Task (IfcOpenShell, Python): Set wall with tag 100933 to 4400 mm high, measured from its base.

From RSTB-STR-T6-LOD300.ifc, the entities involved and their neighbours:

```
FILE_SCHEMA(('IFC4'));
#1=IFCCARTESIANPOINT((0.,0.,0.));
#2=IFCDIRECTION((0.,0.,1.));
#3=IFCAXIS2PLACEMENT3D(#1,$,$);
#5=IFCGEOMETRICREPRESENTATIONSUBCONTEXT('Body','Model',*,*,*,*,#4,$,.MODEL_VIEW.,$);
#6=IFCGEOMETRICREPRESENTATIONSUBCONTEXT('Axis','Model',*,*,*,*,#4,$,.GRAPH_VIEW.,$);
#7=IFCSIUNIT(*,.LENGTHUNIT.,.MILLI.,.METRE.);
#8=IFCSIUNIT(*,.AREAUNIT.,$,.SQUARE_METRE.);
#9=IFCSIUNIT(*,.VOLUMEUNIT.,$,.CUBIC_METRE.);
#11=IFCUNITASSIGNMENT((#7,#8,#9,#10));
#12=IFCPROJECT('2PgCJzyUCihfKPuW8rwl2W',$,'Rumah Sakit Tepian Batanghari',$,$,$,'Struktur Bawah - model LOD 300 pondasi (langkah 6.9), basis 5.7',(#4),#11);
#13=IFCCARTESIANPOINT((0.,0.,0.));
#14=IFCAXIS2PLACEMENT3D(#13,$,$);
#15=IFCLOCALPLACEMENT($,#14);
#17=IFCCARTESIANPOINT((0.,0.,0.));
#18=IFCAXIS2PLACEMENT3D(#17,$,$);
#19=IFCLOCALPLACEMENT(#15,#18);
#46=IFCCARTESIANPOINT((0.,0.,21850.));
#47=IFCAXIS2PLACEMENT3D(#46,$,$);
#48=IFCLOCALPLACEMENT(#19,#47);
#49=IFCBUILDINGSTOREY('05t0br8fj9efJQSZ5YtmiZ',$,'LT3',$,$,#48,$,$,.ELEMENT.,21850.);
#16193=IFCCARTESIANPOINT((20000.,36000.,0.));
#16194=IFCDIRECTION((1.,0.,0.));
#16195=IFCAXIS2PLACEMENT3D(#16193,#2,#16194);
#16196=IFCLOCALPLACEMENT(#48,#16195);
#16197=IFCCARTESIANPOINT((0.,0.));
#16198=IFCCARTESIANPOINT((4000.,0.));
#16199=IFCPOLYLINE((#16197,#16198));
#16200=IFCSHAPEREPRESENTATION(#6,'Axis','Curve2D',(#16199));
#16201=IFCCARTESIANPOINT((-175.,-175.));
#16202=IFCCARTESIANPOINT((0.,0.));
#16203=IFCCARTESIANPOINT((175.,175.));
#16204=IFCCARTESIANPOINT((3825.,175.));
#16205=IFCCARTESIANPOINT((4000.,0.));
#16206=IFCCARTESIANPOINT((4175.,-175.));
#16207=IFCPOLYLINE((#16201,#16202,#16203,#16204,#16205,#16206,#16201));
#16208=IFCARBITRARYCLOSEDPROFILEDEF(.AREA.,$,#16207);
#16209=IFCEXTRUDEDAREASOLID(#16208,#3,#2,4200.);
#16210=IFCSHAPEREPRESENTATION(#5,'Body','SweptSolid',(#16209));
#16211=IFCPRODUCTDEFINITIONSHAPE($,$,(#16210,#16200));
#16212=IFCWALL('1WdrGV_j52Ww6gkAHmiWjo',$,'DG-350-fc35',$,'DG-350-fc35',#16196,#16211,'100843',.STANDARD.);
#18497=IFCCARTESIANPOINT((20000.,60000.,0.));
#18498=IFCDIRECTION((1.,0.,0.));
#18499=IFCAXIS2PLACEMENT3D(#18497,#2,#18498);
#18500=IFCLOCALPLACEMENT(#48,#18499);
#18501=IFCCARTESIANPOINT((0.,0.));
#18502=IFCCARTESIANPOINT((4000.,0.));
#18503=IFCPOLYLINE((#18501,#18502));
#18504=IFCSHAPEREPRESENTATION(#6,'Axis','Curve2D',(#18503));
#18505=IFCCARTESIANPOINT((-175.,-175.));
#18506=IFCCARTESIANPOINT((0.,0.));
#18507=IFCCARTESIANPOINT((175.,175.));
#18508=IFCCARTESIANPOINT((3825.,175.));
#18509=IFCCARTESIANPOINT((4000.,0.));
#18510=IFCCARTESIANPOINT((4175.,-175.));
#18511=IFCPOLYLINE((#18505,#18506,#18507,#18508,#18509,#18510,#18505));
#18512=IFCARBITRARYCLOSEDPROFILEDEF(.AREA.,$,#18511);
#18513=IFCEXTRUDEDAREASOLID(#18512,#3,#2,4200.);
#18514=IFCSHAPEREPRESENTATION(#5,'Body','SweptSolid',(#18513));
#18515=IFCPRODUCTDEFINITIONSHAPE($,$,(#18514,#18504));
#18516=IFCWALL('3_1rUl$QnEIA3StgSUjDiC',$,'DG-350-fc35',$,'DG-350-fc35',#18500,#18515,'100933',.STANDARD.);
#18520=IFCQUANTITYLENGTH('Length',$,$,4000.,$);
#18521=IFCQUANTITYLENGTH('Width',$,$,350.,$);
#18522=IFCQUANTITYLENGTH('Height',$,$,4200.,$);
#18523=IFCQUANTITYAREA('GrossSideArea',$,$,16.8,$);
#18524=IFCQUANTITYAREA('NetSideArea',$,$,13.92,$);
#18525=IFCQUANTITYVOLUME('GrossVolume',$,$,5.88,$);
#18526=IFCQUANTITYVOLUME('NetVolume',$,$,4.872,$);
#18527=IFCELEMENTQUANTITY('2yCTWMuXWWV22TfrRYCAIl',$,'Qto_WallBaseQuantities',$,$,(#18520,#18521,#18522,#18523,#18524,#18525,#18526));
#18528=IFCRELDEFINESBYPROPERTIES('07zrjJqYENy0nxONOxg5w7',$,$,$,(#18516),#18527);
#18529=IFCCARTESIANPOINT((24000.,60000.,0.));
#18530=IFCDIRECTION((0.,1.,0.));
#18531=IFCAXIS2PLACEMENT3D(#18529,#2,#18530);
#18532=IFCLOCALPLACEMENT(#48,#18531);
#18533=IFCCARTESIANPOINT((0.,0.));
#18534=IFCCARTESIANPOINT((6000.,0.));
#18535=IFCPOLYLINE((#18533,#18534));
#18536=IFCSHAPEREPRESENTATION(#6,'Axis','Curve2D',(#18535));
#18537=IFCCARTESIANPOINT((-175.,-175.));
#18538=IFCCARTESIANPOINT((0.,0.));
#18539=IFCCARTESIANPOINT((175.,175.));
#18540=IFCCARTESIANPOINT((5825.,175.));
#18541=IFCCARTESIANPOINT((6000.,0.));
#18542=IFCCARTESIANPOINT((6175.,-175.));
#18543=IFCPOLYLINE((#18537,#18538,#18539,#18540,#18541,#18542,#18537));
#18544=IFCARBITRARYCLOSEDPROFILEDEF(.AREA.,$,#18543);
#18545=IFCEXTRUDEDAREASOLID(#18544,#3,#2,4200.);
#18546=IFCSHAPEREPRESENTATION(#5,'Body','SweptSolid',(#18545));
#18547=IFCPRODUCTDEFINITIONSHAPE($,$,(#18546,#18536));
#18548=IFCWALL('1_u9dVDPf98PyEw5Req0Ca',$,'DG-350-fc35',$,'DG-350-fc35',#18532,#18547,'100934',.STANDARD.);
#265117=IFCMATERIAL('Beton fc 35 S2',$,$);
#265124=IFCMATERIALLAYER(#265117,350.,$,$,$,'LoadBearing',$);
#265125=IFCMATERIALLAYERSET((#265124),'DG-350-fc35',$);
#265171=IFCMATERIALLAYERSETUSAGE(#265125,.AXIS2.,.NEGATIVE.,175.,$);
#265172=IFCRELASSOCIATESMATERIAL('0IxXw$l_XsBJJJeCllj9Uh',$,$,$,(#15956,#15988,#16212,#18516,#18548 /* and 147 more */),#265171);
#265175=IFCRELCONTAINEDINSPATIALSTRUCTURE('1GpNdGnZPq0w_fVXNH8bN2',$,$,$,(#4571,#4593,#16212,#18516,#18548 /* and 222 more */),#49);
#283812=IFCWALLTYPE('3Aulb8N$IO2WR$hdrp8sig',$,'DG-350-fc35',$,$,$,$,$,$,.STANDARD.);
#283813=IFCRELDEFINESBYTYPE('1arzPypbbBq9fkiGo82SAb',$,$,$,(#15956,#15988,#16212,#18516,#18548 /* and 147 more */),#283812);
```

```python
import ifcopenshell
import ifcopenshell.api.pset
import ifcopenshell.geom
import ifcopenshell.util.element
import ifcopenshell.util.representation
import ifcopenshell.util.shape
import ifcopenshell.util.unit

model = ifcopenshell.open("RSTB-STR-T6-LOD300.ifc")
unit_scale = ifcopenshell.util.unit.calculate_unit_scale(model)
area_scale = ifcopenshell.util.unit.calculate_unit_scale(model, "AREAUNIT")
volume_scale = ifcopenshell.util.unit.calculate_unit_scale(model, "VOLUMEUNIT")
settings = ifcopenshell.geom.settings()


def volume(element):
    """Net volume in cubic metres, openings subtracted."""
    shape = ifcopenshell.geom.create_shape(settings, element)
    return ifcopenshell.util.shape.get_volume(shape.geometry)


wall = model.by_id(18516)
before = volume(wall)

body = ifcopenshell.util.representation.get_representation(wall, "Model", "Body")
solid = body.Items[0]
old_height = solid.Depth
solid.Depth = 4.4 / unit_scale
after = volume(wall)
thickness = 0.35  # wall thickness in metres

# Update the stored height, areas and volumes.
qto = model.by_id(ifcopenshell.util.element.get_pset(wall, "Qto_WallBaseQuantities", should_inherit=False)["id"])
ifcopenshell.api.pset.edit_qto(model, qto=qto, properties={
    "Height": solid.Depth,
    "GrossSideArea": ifcopenshell.util.element.get_pset(wall, "Qto_WallBaseQuantities", "GrossSideArea") * solid.Depth / old_height,
    "NetSideArea": after / thickness / area_scale,
    "GrossVolume": ifcopenshell.util.element.get_pset(wall, "Qto_WallBaseQuantities", "GrossVolume") * solid.Depth / old_height,
    "NetVolume": after / volume_scale,
})

print(f"height {old_height:g} -> {solid.Depth:g}, volume {before:.3f} -> {after:.3f} m3")

model.write("RSTB-STR-T6-LOD300_v2.ifc")
```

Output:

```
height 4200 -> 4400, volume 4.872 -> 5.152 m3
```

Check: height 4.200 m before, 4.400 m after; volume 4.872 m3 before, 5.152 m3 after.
